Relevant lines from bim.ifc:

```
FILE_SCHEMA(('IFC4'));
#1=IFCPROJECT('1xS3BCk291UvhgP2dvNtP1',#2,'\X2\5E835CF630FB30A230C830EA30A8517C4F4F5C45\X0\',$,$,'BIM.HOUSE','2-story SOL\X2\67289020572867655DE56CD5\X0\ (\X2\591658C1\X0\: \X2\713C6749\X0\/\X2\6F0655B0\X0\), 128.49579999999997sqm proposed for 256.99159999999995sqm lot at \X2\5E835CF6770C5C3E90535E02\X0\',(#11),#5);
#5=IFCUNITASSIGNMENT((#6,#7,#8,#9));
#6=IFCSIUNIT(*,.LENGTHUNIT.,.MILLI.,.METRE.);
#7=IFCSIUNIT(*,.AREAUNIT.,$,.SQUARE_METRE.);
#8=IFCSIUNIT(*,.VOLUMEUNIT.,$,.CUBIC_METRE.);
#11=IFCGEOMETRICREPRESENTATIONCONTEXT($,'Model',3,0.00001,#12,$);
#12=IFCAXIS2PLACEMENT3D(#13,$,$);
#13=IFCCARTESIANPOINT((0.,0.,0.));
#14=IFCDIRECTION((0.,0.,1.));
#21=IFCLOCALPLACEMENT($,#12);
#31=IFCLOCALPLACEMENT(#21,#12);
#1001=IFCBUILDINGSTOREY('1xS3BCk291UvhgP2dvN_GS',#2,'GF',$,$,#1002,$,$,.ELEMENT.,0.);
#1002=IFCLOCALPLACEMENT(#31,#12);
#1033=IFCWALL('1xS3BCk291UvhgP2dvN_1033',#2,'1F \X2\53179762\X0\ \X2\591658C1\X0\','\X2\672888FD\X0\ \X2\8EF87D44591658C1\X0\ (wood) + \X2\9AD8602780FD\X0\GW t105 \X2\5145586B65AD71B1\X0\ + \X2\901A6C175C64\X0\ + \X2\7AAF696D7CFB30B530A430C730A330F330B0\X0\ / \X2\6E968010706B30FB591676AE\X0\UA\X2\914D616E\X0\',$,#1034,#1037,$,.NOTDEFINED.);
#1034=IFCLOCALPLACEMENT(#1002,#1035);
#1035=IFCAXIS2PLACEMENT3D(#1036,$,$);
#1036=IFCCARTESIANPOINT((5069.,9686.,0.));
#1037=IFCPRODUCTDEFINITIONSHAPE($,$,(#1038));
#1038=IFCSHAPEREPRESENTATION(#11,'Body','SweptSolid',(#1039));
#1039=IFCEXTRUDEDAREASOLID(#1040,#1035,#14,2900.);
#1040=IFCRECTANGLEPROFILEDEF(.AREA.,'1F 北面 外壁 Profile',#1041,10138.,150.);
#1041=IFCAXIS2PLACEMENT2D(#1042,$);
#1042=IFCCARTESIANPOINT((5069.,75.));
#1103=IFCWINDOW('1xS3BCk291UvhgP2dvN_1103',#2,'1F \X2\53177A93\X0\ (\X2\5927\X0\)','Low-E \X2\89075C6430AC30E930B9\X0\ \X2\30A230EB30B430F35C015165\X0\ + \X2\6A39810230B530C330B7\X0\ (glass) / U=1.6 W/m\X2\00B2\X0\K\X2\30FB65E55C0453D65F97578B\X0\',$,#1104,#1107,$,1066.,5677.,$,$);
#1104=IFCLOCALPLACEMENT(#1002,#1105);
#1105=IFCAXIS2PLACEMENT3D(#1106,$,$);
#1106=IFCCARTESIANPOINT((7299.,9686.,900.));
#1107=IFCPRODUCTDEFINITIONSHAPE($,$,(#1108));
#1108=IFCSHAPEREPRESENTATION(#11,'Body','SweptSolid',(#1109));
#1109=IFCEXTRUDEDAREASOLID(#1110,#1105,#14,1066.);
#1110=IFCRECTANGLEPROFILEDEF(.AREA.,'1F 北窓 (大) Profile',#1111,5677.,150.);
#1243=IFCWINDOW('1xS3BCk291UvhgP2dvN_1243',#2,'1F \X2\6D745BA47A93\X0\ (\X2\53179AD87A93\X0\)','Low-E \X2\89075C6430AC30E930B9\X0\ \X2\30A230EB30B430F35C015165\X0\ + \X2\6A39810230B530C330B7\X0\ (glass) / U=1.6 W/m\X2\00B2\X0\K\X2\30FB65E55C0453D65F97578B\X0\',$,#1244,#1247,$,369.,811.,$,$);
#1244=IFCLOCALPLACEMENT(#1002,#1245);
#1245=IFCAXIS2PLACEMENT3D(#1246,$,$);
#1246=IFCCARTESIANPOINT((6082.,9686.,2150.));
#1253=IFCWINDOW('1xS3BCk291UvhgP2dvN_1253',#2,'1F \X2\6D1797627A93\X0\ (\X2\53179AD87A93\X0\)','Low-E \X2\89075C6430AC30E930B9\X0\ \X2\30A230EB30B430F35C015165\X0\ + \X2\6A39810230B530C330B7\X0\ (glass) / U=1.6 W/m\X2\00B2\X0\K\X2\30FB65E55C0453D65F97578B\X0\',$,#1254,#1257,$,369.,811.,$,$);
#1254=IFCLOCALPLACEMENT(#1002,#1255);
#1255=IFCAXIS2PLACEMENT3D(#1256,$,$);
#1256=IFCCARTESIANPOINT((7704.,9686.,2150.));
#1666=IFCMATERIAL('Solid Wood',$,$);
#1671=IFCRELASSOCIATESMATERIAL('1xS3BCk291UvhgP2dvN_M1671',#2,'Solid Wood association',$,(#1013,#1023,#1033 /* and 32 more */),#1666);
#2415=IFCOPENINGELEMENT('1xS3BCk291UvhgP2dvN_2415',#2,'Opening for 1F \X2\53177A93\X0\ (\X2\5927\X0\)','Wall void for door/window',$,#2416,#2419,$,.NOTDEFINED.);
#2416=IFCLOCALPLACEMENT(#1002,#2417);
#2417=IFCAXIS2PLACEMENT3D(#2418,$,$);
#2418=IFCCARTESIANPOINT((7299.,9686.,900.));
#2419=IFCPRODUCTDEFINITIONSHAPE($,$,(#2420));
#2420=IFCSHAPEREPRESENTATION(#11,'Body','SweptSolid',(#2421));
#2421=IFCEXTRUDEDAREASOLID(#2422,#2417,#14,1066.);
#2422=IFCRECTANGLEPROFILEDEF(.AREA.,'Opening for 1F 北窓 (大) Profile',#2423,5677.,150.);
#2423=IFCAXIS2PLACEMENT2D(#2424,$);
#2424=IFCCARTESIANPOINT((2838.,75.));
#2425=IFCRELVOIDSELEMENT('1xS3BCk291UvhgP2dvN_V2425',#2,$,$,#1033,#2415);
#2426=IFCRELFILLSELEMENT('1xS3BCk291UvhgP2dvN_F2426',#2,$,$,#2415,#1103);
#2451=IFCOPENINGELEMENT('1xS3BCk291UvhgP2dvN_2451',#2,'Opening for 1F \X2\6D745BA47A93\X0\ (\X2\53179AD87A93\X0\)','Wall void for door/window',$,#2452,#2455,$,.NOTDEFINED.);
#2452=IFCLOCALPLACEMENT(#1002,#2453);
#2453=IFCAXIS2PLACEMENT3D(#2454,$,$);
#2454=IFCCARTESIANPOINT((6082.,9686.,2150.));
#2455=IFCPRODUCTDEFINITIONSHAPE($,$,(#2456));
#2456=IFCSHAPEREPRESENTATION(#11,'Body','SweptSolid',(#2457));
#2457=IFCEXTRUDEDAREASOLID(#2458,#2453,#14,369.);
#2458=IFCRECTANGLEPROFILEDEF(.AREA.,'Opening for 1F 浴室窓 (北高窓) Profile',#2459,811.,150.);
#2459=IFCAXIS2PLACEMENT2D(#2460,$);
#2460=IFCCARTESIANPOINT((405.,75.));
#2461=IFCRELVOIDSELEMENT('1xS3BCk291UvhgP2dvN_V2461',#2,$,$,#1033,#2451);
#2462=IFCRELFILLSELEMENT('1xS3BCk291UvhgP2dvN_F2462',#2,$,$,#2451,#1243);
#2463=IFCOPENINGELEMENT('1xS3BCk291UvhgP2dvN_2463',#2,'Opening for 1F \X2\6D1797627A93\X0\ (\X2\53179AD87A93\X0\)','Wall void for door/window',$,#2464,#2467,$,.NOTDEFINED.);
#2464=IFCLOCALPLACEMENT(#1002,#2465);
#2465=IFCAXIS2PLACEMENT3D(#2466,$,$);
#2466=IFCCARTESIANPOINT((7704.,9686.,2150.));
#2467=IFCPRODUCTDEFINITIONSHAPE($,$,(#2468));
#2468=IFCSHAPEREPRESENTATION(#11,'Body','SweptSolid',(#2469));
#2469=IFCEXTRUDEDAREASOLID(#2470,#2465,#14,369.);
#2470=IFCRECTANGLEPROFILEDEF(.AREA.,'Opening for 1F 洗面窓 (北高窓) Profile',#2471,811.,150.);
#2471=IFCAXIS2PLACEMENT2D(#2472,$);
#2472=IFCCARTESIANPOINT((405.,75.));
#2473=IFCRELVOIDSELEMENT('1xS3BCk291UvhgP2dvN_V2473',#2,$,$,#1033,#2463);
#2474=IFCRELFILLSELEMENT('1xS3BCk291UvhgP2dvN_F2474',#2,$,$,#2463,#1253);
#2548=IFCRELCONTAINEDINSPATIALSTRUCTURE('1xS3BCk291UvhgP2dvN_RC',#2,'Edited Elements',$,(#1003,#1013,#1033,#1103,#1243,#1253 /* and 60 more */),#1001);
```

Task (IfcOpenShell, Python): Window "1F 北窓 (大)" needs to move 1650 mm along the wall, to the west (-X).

```python
import ifcopenshell
import ifcopenshell.api.geometry
import ifcopenshell.util.placement
import ifcopenshell.util.unit

model = ifcopenshell.open("bim.ifc")
unit_scale = ifcopenshell.util.unit.calculate_unit_scale(model)

window = model.by_guid("1xS3BCk291UvhgP2dvN_1103")
opening = window.FillsVoids[0].RelatingOpeningElement
wall = opening.VoidsElements[0].RelatingBuildingElement

wall_matrix = ifcopenshell.util.placement.get_local_placement(wall.ObjectPlacement)
shift = wall_matrix[:3, 0] * -1.65 / unit_scale
before = ifcopenshell.util.placement.get_local_placement(window.ObjectPlacement)[:3, 3].copy()

# The window is not placed relative to its opening, so move both.
for product in (opening, window):
    matrix = ifcopenshell.util.placement.get_local_placement(product.ObjectPlacement)
    matrix[:3, 3] += shift
    ifcopenshell.api.geometry.edit_object_placement(model, product=product, matrix=matrix, is_si=False)

after = ifcopenshell.util.placement.get_local_placement(window.ObjectPlacement)[:3, 3]
print("window moved by", (after - before).round(3) + 0.0)

model.write("bim-out.ifc")
```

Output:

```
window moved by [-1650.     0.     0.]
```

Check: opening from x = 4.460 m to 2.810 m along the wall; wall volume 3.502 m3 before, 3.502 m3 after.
